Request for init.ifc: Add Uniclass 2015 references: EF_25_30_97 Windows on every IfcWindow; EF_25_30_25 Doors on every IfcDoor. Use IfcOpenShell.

First a look at what the model holds.

```python
import ifcopenshell

model = ifcopenshell.open("init.ifc")
print(model.schema)
print("classifications:", [c.Name for c in model.by_type("IfcClassification")])
for ifc_class in ("IfcDoor", "IfcRoof", "IfcStair", "IfcWall", "IfcWindow"):
    print(ifc_class, len(model.by_type(ifc_class)))
```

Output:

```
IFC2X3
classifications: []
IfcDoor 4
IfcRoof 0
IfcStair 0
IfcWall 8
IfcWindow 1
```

```python
import ifcopenshell
import ifcopenshell.api.classification

model = ifcopenshell.open("init.ifc")

# IFC2X3 requires Source and Edition and has no link from the project to the system.
system = model.create_entity("IfcClassification", Source="NBS", Edition="2015", Name="Uniclass 2015")

codes = {
    "IfcWindow": ("EF_25_30_97", "Windows"),
    "IfcDoor": ("EF_25_30_25", "Doors"),
}
for ifc_class, (code, name) in codes.items():
    products = model.by_type(ifc_class)
    ifcopenshell.api.classification.add_reference(
        model, products=products, classification=system, identification=code, name=name
    )
    print(code, len(products))

model.write("init_rev.ifc")
```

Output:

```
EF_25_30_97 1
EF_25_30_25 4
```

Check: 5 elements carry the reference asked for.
